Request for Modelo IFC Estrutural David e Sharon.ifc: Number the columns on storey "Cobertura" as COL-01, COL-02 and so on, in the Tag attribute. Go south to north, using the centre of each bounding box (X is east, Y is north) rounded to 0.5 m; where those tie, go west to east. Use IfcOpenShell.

First a look at what the model holds.

```python
import ifcopenshell
import ifcopenshell.util.element
import ifcopenshell.util.placement

model = ifcopenshell.open("Modelo IFC Estrutural David e Sharon.ifc")
print(model.schema)
storey = next(s for s in model.by_type("IfcBuildingStorey") if s.Name == "Cobertura")
columns = [e for e in ifcopenshell.util.element.get_decomposition(storey) if e.is_a("IfcColumn")]
for e in sorted(columns, key=lambda e: e.id()):
    origin = ifcopenshell.util.placement.get_local_placement(e.ObjectPlacement)[:3, 3]
    print(e.id(), e.Tag, e.Name, origin.round(2) + 0.0, sep=" | ")
```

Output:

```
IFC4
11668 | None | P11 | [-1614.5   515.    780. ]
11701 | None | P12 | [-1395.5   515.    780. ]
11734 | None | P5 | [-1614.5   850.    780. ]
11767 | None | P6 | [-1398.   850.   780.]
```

```python
import ifcopenshell
import ifcopenshell.geom
import ifcopenshell.util.element
import ifcopenshell.util.shape

model = ifcopenshell.open("Modelo IFC Estrutural David e Sharon.ifc")
settings = ifcopenshell.geom.settings()
settings.set("use-world-coords", True)


def centre(element):
    shape = ifcopenshell.geom.create_shape(settings, element)
    return ifcopenshell.util.shape.get_bbox_centroid(shape.geometry)


storey = next(s for s in model.by_type("IfcBuildingStorey") if s.Name == "Cobertura")
columns = [e for e in ifcopenshell.util.element.get_decomposition(storey) if e.is_a("IfcColumn")]

# Insertion points can sit at a corner or the storey origin, so sort by the geometry (in metres).
centres = {e: centre(e) for e in columns}
columns.sort(key=lambda e: (round(centres[e][1] / 0.5), centres[e][0]))

for i, e in enumerate(columns, start=1):
    number = f"COL-{i:02d}"
    e.Tag = number
    print(e.id(), number)

model.write("Modelo IFC Estrutural David e Sharon_v2.ifc")
```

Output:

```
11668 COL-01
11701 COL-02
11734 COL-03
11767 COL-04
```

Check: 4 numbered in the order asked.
